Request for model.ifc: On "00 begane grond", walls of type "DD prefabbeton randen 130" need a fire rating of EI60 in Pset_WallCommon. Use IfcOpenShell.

First a look at what the model holds.

```python
import ifcopenshell
import ifcopenshell.util.element

model = ifcopenshell.open("model.ifc")
print(model.schema)
storey = next(s for s in model.by_type("IfcBuildingStorey") if s.Name == "00 begane grond")
walls = [e for e in ifcopenshell.util.element.get_decomposition(storey) if e.is_a("IfcWall")]
seen = {}
for e in walls:
    element_type = ifcopenshell.util.element.get_type(e)
    key = (element_type.Name if element_type != e and element_type else None, ifcopenshell.util.element.get_pset(e, "Pset_WallCommon", "FireRating"))
    seen[key] = seen.get(key, 0) + 1
for (name, value), count in sorted(seen.items(), key=str):
    print(count, "x", name, "|", value)
```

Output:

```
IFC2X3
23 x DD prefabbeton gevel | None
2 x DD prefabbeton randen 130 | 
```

```python
import ifcopenshell
import ifcopenshell.api.pset
import ifcopenshell.util.element

model = ifcopenshell.open("model.ifc")

storey = next(s for s in model.by_type("IfcBuildingStorey") if s.Name == "00 begane grond")
walls = [e for e in ifcopenshell.util.element.get_decomposition(storey) if e.is_a("IfcWall")]

count = 0
for e in walls:
    element_type = ifcopenshell.util.element.get_type(e)
    if element_type in (None, e) or element_type.Name != "DD prefabbeton randen 130":
        continue
    # add_pset returns the element's existing set when there is one.
    pset = ifcopenshell.api.pset.add_pset(model, product=e, name="Pset_WallCommon")
    ifcopenshell.api.pset.edit_pset(model, pset=pset, properties={"FireRating": "EI60"})
    count += 1

print(count, "walls updated")

model.write("model_edited.ifc")
```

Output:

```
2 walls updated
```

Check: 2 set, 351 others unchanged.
